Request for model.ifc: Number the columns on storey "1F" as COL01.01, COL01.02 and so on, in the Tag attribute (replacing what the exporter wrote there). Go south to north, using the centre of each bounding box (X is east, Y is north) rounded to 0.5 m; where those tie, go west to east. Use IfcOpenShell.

First a look at what the model holds.

```python
import ifcopenshell
import ifcopenshell.util.element
import ifcopenshell.util.placement

model = ifcopenshell.open("model.ifc")
print(model.schema)
storey = next(s for s in model.by_type("IfcBuildingStorey") if s.Name == "1F")
columns = [e for e in ifcopenshell.util.element.get_decomposition(storey) if e.is_a("IfcColumn")]
for e in sorted(columns, key=lambda e: e.id()):
    origin = ifcopenshell.util.placement.get_local_placement(e.ObjectPlacement)[:3, 3]
    print(e.id(), e.Tag, e.Name, origin.round(2) + 0.0, sep=" | ")
```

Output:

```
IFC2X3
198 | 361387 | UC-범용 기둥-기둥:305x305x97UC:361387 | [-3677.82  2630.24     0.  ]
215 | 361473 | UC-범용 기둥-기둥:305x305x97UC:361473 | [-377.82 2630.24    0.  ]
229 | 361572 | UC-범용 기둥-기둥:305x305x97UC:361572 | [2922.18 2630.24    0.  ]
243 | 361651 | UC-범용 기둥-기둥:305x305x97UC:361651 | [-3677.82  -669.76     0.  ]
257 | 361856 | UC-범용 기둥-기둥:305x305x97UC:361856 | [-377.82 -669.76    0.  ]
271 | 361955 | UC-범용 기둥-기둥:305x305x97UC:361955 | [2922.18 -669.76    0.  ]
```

```python
import ifcopenshell
import ifcopenshell.geom
import ifcopenshell.util.element
import ifcopenshell.util.shape

model = ifcopenshell.open("model.ifc")
settings = ifcopenshell.geom.settings()
settings.set("use-world-coords", True)


def centre(element):
    shape = ifcopenshell.geom.create_shape(settings, element)
    return ifcopenshell.util.shape.get_bbox_centroid(shape.geometry)


storey = next(s for s in model.by_type("IfcBuildingStorey") if s.Name == "1F")
columns = [e for e in ifcopenshell.util.element.get_decomposition(storey) if e.is_a("IfcColumn")]

# Insertion points can sit at a corner or the storey origin, so sort by the geometry (in metres).
centres = {e: centre(e) for e in columns}
columns.sort(key=lambda e: (round(centres[e][1] / 0.5), centres[e][0]))

for i, e in enumerate(columns, start=1):
    number = f"COL01.{i:02d}"
    e.Tag = number
    print(e.id(), number)

model.write("model-out.ifc")
```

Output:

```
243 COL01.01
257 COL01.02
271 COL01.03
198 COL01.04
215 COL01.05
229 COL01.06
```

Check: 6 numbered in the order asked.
